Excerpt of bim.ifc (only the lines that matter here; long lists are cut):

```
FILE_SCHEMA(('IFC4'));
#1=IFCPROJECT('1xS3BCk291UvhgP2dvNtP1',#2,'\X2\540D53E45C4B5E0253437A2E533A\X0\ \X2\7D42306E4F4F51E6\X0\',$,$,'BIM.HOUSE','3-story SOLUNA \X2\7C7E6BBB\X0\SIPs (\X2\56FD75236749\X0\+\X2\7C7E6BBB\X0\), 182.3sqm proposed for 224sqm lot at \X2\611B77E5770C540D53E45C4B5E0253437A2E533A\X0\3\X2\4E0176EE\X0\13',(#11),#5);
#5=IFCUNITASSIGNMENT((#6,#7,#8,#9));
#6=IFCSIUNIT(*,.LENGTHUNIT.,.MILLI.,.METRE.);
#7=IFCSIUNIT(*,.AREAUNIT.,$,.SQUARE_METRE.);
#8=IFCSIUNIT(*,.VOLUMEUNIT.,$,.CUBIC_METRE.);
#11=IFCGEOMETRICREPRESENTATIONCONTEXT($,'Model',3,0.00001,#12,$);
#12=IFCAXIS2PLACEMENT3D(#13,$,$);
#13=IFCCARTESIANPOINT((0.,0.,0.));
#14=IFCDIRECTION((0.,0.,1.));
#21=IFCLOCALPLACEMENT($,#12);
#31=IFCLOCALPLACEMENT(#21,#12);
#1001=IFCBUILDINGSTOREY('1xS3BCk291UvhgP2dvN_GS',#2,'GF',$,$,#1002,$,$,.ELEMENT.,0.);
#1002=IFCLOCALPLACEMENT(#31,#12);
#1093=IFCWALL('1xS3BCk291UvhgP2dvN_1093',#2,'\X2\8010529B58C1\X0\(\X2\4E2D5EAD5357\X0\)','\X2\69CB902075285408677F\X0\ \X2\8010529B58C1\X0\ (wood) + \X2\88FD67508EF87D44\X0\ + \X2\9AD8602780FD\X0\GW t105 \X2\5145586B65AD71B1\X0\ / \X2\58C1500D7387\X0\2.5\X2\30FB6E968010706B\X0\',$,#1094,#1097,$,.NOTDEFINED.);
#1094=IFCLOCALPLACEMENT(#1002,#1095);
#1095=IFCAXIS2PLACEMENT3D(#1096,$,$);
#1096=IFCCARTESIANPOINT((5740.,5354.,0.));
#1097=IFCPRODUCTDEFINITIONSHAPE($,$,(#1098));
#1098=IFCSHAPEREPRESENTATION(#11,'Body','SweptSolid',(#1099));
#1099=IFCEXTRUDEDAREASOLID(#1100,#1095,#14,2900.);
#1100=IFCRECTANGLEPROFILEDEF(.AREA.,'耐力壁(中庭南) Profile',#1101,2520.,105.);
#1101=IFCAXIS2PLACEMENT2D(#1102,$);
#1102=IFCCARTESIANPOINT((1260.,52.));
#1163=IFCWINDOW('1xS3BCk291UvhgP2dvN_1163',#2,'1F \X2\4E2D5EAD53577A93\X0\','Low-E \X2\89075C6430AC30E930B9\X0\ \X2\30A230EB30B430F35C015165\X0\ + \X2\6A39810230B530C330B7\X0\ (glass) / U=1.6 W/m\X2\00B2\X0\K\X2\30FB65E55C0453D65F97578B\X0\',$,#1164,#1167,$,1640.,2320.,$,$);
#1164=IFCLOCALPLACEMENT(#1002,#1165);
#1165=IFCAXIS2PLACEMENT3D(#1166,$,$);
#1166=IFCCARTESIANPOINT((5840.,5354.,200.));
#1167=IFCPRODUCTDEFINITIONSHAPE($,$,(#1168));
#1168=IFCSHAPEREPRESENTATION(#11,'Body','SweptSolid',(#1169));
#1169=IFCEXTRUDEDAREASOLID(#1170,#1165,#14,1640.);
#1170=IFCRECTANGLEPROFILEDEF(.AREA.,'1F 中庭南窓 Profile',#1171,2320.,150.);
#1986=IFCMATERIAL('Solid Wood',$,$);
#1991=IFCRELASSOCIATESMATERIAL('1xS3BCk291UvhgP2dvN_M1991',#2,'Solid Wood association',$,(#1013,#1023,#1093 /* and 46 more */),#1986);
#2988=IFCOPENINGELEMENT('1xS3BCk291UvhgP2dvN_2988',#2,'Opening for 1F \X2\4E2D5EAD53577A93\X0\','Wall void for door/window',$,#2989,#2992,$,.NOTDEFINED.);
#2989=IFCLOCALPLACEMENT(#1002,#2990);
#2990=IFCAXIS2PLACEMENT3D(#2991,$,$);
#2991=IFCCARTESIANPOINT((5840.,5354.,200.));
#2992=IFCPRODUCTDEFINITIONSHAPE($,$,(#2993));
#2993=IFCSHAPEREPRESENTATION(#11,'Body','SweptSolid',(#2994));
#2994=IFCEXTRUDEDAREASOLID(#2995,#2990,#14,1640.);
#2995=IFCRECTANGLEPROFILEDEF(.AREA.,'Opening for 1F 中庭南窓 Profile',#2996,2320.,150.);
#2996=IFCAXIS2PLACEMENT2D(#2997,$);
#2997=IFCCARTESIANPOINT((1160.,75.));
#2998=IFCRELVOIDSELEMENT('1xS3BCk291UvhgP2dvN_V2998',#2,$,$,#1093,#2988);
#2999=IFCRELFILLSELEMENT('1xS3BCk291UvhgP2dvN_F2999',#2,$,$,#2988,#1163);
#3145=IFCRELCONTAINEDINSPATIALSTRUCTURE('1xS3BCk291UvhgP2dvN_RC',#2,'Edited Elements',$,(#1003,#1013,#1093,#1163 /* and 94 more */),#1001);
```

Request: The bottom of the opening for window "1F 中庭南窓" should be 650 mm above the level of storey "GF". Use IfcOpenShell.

```python
import numpy as np
import ifcopenshell
import ifcopenshell.api.geometry
import ifcopenshell.geom
import ifcopenshell.util.element
import ifcopenshell.util.placement
import ifcopenshell.util.shape
import ifcopenshell.util.unit

model = ifcopenshell.open("bim.ifc")
unit_scale = ifcopenshell.util.unit.calculate_unit_scale(model)

window = model.by_guid("1xS3BCk291UvhgP2dvN_1163")
opening = window.FillsVoids[0].RelatingOpeningElement
storey = ifcopenshell.util.element.get_container(window, ifc_class="IfcBuildingStorey")
level = ifcopenshell.util.placement.get_local_placement(storey.ObjectPlacement)[2, 3]

# The opening's origin need not be at the sill, so measure its lowest point.
shape = ifcopenshell.geom.create_shape(ifcopenshell.geom.settings(), opening)
bottom = ifcopenshell.util.shape.get_shape_bottom_elevation(shape, shape.geometry) / unit_scale
dz = level + 650.0 - bottom

shift = np.array([0.0, 0.0, dz])
# The window is not placed relative to its opening, so move both.
for product in (opening, window):
    matrix = ifcopenshell.util.placement.get_local_placement(product.ObjectPlacement)
    matrix[:3, 3] += shift
    ifcopenshell.api.geometry.edit_object_placement(model, product=product, matrix=matrix, is_si=False)

print(f"moved by {dz * unit_scale:+.3f} m")

model.write("bim_updated.ifc")
```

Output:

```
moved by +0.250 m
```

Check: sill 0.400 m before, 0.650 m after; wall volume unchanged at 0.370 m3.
